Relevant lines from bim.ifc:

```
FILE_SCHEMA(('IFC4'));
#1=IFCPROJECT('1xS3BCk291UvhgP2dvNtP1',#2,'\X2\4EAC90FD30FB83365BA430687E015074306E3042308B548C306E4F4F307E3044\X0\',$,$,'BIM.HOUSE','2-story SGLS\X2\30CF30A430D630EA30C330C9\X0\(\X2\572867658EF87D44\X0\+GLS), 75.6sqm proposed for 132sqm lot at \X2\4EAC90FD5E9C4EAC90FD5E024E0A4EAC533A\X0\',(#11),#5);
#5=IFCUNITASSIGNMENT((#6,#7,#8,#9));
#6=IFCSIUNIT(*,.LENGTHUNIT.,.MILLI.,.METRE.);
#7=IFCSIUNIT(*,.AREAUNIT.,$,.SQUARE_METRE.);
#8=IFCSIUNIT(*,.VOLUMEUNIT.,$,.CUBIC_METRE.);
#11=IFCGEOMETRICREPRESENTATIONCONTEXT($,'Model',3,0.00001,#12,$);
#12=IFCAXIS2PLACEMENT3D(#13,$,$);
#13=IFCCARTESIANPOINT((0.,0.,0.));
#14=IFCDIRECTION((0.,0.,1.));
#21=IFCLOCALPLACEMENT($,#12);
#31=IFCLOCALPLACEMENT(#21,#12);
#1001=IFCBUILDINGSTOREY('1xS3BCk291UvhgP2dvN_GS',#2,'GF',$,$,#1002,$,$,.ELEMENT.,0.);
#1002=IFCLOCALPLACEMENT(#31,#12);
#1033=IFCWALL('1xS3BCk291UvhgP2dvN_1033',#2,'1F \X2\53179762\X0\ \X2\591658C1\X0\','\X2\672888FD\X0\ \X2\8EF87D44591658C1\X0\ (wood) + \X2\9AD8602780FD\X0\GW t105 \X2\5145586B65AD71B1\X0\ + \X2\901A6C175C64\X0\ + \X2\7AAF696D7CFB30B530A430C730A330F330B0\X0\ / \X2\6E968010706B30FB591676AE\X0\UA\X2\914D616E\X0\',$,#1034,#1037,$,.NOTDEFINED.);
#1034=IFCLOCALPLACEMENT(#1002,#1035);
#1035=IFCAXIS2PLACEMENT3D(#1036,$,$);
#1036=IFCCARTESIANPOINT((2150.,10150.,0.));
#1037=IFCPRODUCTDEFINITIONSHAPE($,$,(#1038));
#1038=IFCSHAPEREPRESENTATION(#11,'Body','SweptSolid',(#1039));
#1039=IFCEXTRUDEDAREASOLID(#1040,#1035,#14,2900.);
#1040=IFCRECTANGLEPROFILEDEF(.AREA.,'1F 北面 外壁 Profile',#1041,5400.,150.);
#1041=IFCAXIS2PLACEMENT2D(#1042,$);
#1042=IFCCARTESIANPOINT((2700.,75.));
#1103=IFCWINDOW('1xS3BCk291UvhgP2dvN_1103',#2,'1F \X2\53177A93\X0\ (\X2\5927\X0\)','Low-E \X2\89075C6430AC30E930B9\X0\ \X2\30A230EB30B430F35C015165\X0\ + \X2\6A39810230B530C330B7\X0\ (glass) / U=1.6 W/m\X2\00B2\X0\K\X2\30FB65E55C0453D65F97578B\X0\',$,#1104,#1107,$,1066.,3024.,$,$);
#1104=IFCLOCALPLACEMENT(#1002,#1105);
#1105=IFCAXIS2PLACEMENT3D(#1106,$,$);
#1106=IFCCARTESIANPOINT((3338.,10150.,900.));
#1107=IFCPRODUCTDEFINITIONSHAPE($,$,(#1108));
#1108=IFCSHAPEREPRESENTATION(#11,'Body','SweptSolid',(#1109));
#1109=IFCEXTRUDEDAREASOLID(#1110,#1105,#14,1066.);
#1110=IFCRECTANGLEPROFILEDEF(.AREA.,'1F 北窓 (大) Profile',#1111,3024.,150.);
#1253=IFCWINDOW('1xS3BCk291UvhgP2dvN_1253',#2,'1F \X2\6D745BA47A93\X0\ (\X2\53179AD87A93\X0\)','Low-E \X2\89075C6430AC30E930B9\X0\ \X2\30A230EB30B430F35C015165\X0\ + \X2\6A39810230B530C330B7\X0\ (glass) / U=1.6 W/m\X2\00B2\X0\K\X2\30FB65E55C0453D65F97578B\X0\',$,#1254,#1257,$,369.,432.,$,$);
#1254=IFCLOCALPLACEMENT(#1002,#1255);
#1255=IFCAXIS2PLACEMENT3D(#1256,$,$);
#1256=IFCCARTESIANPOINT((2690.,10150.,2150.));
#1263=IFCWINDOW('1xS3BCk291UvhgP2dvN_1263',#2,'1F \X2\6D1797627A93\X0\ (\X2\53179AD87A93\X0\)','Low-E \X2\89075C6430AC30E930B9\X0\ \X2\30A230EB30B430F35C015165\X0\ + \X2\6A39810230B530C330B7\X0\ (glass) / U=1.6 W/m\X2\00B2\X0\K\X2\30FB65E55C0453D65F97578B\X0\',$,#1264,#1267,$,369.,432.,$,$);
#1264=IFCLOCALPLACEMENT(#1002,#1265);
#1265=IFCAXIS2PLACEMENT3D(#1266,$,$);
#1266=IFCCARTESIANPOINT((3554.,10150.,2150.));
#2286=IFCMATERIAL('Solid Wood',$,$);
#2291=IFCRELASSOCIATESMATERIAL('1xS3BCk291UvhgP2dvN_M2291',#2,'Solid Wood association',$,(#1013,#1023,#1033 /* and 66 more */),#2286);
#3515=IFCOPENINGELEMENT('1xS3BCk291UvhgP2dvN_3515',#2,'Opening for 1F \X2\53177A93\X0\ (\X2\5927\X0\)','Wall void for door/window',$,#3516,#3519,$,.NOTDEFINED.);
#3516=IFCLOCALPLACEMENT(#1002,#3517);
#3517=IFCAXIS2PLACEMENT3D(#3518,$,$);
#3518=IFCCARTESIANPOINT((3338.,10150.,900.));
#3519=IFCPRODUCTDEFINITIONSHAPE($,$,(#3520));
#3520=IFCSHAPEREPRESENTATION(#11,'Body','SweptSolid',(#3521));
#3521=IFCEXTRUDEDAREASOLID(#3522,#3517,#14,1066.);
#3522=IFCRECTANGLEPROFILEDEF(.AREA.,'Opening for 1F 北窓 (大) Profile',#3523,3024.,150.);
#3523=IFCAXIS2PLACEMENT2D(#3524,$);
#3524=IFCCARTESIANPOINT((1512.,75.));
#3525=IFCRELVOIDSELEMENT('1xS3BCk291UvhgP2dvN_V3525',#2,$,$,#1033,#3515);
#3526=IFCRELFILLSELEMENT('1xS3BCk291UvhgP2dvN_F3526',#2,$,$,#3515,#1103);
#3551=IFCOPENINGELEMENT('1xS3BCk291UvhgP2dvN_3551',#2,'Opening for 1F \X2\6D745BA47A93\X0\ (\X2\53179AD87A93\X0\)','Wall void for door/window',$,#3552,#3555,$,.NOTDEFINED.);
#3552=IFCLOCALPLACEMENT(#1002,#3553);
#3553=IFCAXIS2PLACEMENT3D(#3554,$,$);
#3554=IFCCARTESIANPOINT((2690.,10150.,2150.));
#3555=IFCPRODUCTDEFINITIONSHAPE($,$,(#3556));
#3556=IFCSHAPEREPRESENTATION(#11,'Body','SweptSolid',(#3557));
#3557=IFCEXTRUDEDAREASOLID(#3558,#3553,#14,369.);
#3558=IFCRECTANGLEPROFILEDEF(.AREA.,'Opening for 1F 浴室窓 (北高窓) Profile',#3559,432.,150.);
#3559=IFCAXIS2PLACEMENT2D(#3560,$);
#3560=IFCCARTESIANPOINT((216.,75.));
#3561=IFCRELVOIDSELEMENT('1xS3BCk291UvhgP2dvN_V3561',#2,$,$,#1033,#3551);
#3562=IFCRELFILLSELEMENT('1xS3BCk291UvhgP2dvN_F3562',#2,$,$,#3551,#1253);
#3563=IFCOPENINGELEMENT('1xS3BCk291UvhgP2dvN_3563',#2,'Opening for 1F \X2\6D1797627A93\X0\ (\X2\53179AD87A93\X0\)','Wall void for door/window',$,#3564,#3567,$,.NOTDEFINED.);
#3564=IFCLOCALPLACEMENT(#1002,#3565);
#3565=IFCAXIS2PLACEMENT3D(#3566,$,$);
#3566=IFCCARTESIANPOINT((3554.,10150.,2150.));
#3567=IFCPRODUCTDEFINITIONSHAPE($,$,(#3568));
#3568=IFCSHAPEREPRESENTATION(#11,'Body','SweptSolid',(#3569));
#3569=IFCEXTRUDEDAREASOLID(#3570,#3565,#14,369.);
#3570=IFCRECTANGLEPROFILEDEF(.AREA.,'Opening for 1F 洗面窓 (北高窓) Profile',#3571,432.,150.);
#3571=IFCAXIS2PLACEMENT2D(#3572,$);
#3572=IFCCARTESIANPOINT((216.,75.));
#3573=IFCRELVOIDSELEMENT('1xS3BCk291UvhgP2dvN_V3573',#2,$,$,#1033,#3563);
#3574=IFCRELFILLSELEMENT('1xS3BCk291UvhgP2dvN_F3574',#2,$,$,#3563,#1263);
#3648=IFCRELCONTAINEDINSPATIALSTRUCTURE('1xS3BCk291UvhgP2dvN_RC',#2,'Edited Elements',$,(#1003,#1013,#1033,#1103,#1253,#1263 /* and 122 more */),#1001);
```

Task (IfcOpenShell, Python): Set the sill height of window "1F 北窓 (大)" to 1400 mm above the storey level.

```python
import numpy as np
import ifcopenshell
import ifcopenshell.api.geometry
import ifcopenshell.geom
import ifcopenshell.util.element
import ifcopenshell.util.placement
import ifcopenshell.util.shape
import ifcopenshell.util.unit

model = ifcopenshell.open("bim.ifc")
unit_scale = ifcopenshell.util.unit.calculate_unit_scale(model)

window = model.by_guid("1xS3BCk291UvhgP2dvN_1103")
opening = window.FillsVoids[0].RelatingOpeningElement
storey = ifcopenshell.util.element.get_container(window, ifc_class="IfcBuildingStorey")
level = ifcopenshell.util.placement.get_local_placement(storey.ObjectPlacement)[2, 3]

# The opening's origin need not be at the sill, so measure its lowest point.
shape = ifcopenshell.geom.create_shape(ifcopenshell.geom.settings(), opening)
bottom = ifcopenshell.util.shape.get_shape_bottom_elevation(shape, shape.geometry) / unit_scale
dz = level + 1.4 / unit_scale - bottom

shift = np.array([0.0, 0.0, dz])
# The window is not placed relative to its opening, so move both.
for product in (opening, window):
    matrix = ifcopenshell.util.placement.get_local_placement(product.ObjectPlacement)
    matrix[:3, 3] += shift
    ifcopenshell.api.geometry.edit_object_placement(model, product=product, matrix=matrix, is_si=False)

print(f"moved by {dz * unit_scale:+.3f} m")

model.write("bim_edited.ifc")
```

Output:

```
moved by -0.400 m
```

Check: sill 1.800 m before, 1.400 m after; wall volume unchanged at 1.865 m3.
